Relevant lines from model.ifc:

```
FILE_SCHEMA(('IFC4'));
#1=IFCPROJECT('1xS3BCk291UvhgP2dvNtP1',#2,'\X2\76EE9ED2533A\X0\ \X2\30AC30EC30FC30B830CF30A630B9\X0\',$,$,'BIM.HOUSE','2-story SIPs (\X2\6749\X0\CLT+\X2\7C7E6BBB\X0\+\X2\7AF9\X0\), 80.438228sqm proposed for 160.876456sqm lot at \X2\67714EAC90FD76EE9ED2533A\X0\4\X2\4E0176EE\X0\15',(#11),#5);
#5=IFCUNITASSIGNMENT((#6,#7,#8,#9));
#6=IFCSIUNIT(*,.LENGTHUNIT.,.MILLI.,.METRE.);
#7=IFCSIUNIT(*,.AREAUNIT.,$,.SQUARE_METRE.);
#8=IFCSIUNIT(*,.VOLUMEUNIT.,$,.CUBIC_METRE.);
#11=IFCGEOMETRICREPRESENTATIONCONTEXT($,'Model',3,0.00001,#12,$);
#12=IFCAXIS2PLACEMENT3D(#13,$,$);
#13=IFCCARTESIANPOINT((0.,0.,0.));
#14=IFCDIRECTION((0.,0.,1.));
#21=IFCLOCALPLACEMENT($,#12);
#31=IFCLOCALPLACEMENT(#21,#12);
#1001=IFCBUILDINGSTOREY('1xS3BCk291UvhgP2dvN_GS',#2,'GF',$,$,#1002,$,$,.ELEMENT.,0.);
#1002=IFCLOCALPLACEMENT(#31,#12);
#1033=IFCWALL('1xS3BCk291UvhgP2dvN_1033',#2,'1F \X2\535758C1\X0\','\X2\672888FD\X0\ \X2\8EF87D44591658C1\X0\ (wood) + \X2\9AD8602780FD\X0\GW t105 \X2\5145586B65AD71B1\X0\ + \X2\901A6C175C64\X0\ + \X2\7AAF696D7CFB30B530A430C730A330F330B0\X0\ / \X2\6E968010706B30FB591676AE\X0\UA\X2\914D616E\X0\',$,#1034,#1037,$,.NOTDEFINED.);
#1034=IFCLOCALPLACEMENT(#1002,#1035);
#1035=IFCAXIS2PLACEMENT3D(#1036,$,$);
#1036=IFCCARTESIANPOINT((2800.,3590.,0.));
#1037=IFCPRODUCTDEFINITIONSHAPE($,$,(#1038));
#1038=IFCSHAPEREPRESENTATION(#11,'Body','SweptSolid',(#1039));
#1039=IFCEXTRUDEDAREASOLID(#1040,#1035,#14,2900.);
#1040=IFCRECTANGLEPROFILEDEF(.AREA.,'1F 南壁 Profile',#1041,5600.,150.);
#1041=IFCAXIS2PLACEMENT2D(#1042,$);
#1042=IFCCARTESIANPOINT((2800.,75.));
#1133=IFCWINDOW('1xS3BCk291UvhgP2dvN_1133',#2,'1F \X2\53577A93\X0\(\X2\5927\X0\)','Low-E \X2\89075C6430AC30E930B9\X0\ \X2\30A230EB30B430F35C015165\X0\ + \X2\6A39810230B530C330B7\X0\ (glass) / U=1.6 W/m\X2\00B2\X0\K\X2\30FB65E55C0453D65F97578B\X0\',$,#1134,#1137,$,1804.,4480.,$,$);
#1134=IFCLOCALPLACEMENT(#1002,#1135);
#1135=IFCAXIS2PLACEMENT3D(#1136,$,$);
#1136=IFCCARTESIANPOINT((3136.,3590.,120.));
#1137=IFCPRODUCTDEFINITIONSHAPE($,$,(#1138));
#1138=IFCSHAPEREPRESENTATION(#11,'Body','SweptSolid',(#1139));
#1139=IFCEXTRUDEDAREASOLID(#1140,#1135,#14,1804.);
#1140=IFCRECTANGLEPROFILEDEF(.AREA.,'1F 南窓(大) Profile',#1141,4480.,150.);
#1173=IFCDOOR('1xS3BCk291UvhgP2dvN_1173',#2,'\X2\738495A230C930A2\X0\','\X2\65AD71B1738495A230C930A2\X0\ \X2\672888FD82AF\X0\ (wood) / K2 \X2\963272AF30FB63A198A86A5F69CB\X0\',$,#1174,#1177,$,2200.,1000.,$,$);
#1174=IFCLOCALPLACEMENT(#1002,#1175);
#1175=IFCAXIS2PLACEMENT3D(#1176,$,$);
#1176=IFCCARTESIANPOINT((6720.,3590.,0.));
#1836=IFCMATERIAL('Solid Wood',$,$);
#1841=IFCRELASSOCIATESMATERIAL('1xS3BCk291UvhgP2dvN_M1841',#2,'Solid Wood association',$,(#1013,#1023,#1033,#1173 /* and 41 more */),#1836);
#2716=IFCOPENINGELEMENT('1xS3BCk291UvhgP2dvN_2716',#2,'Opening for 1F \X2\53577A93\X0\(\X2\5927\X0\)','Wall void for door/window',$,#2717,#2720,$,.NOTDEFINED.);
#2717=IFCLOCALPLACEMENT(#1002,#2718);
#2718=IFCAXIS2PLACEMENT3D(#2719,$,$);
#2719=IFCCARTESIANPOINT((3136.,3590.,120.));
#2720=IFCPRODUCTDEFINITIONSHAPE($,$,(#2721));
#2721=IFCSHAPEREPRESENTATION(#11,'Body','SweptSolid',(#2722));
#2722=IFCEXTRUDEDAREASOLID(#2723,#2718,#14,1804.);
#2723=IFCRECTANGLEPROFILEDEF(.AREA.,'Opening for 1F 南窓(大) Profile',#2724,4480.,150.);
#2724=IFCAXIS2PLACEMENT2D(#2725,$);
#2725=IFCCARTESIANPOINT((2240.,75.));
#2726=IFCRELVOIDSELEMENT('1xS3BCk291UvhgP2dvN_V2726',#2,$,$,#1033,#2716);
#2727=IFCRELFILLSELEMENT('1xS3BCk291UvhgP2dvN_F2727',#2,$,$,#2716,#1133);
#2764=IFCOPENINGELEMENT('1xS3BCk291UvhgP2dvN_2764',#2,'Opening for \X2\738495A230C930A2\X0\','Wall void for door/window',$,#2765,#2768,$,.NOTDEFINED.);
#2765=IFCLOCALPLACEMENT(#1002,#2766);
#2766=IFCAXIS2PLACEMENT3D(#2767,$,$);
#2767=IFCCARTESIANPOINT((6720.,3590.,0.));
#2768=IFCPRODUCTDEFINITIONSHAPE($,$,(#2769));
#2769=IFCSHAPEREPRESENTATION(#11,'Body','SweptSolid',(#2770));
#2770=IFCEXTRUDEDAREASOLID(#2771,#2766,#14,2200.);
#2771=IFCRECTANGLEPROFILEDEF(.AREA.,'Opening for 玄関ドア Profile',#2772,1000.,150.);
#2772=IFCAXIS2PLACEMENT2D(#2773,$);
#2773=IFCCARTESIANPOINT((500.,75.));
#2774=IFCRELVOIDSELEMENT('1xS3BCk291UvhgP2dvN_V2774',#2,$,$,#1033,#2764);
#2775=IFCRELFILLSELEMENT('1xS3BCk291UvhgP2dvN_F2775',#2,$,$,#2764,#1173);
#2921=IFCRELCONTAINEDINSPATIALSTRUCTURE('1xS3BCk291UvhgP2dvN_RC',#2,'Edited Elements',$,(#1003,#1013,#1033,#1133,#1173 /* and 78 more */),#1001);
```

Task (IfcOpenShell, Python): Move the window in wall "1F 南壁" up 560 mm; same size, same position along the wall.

```python
import numpy as np
import ifcopenshell
import ifcopenshell.api.geometry
import ifcopenshell.util.placement
import ifcopenshell.util.unit

model = ifcopenshell.open("model.ifc")
unit_scale = ifcopenshell.util.unit.calculate_unit_scale(model)

window = model.by_guid("1xS3BCk291UvhgP2dvN_1133")
opening = window.FillsVoids[0].RelatingOpeningElement
dz = 0.56 / unit_scale

shift = np.array([0.0, 0.0, dz])
# The window is not placed relative to its opening, so move both.
for product in (opening, window):
    matrix = ifcopenshell.util.placement.get_local_placement(product.ObjectPlacement)
    matrix[:3, 3] += shift
    ifcopenshell.api.geometry.edit_object_placement(model, product=product, matrix=matrix, is_si=False)

print(f"moved by {dz * unit_scale:+.3f} m")

model.write("model_edited.ifc")
```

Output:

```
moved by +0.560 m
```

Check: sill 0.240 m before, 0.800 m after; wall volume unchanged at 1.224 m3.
